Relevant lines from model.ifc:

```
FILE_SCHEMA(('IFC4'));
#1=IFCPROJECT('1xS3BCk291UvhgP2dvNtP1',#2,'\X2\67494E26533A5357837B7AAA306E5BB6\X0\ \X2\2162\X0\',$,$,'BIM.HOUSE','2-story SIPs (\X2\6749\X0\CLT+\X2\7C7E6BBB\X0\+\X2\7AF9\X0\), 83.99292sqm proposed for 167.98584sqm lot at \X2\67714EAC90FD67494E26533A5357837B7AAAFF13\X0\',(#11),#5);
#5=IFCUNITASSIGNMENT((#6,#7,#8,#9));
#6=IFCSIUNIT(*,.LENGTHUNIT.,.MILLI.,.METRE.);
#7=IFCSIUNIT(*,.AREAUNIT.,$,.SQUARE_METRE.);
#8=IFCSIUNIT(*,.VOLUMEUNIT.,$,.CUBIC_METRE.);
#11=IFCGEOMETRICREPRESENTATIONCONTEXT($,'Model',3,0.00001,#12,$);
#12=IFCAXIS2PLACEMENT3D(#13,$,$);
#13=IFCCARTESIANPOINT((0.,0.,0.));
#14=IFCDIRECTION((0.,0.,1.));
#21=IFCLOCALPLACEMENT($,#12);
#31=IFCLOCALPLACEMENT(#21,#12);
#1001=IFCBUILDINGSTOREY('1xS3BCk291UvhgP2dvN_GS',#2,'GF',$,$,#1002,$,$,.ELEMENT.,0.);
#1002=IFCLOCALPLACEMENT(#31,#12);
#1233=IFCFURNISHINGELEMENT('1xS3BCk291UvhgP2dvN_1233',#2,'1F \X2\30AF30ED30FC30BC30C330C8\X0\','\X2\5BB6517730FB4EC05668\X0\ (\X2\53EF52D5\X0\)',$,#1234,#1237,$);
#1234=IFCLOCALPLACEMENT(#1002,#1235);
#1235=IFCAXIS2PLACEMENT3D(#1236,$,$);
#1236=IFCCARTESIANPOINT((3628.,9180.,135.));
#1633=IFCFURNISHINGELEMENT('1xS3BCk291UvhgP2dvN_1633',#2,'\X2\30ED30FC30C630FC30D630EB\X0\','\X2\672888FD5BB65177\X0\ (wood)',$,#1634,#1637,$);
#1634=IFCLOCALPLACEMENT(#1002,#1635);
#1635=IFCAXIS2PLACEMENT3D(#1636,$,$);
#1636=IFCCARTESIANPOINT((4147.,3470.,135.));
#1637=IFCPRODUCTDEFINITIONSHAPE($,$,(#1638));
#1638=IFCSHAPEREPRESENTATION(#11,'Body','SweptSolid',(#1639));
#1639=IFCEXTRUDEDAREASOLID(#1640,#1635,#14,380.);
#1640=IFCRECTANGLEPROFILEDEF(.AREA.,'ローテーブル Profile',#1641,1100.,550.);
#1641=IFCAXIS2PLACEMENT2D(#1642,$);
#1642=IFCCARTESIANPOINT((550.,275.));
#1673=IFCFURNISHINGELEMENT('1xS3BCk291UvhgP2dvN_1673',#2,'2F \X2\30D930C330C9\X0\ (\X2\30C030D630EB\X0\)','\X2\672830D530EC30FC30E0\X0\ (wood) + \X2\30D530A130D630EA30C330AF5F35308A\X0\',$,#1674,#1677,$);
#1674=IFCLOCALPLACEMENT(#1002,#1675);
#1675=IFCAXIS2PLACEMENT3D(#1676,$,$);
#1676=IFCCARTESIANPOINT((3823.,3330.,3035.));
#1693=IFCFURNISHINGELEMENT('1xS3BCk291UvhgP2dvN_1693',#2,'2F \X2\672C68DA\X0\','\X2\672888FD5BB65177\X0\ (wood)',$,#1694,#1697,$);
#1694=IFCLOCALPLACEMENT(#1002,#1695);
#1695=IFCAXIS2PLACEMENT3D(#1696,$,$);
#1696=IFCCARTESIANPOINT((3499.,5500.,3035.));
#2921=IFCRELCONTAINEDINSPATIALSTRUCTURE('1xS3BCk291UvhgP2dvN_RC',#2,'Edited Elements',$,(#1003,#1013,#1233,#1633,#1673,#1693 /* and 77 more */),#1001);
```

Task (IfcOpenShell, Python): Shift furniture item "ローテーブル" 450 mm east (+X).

```python
import ifcopenshell
import ifcopenshell.api.geometry
import ifcopenshell.util.placement

model = ifcopenshell.open("model.ifc")

item = model.by_id(1633)
matrix = ifcopenshell.util.placement.get_local_placement(item.ObjectPlacement)
matrix[0, 3] += 450.0
ifcopenshell.api.geometry.edit_object_placement(model, product=item, matrix=matrix, is_si=False)

print(ifcopenshell.util.placement.get_local_placement(item.ObjectPlacement).round(3) + 0.0)

model.write("model_rev.ifc")
```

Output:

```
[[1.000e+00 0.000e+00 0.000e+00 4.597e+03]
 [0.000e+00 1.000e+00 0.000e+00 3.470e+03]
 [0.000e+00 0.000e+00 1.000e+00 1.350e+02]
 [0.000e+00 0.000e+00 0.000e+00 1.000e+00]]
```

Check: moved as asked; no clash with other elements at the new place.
